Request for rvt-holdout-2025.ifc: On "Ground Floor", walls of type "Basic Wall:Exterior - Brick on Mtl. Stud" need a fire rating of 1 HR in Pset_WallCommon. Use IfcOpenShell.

First a look at what the model holds.

```python
import ifcopenshell
import ifcopenshell.util.element

model = ifcopenshell.open("rvt-holdout-2025.ifc")
print(model.schema)
storey = next(s for s in model.by_type("IfcBuildingStorey") if s.Name == "Ground Floor")
walls = [e for e in ifcopenshell.util.element.get_decomposition(storey) if e.is_a("IfcWall")]
seen = {}
for e in walls:
    element_type = ifcopenshell.util.element.get_type(e)
    key = (element_type.Name if element_type != e and element_type else None, ifcopenshell.util.element.get_pset(e, "Pset_WallCommon", "FireRating"))
    seen[key] = seen.get(key, 0) + 1
for (name, value), count in sorted(seen.items(), key=str):
    print(count, "x", name, "|", value)
```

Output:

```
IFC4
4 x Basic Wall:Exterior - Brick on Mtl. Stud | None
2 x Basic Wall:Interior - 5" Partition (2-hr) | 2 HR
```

```python
import ifcopenshell
import ifcopenshell.api.pset
import ifcopenshell.util.element

model = ifcopenshell.open("rvt-holdout-2025.ifc")

storey = next(s for s in model.by_type("IfcBuildingStorey") if s.Name == "Ground Floor")
walls = [e for e in ifcopenshell.util.element.get_decomposition(storey) if e.is_a("IfcWall")]

count = 0
for e in walls:
    element_type = ifcopenshell.util.element.get_type(e)
    if element_type in (None, e) or element_type.Name != "Basic Wall:Exterior - Brick on Mtl. Stud":
        continue
    # add_pset returns the element's existing set when there is one.
    pset = ifcopenshell.api.pset.add_pset(model, product=e, name="Pset_WallCommon")
    ifcopenshell.api.pset.edit_pset(model, pset=pset, properties={"FireRating": "1 HR"})
    count += 1

print(count, "walls updated")

model.write("rvt-holdout-2025_updated.ifc")
```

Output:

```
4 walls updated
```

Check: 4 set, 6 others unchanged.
